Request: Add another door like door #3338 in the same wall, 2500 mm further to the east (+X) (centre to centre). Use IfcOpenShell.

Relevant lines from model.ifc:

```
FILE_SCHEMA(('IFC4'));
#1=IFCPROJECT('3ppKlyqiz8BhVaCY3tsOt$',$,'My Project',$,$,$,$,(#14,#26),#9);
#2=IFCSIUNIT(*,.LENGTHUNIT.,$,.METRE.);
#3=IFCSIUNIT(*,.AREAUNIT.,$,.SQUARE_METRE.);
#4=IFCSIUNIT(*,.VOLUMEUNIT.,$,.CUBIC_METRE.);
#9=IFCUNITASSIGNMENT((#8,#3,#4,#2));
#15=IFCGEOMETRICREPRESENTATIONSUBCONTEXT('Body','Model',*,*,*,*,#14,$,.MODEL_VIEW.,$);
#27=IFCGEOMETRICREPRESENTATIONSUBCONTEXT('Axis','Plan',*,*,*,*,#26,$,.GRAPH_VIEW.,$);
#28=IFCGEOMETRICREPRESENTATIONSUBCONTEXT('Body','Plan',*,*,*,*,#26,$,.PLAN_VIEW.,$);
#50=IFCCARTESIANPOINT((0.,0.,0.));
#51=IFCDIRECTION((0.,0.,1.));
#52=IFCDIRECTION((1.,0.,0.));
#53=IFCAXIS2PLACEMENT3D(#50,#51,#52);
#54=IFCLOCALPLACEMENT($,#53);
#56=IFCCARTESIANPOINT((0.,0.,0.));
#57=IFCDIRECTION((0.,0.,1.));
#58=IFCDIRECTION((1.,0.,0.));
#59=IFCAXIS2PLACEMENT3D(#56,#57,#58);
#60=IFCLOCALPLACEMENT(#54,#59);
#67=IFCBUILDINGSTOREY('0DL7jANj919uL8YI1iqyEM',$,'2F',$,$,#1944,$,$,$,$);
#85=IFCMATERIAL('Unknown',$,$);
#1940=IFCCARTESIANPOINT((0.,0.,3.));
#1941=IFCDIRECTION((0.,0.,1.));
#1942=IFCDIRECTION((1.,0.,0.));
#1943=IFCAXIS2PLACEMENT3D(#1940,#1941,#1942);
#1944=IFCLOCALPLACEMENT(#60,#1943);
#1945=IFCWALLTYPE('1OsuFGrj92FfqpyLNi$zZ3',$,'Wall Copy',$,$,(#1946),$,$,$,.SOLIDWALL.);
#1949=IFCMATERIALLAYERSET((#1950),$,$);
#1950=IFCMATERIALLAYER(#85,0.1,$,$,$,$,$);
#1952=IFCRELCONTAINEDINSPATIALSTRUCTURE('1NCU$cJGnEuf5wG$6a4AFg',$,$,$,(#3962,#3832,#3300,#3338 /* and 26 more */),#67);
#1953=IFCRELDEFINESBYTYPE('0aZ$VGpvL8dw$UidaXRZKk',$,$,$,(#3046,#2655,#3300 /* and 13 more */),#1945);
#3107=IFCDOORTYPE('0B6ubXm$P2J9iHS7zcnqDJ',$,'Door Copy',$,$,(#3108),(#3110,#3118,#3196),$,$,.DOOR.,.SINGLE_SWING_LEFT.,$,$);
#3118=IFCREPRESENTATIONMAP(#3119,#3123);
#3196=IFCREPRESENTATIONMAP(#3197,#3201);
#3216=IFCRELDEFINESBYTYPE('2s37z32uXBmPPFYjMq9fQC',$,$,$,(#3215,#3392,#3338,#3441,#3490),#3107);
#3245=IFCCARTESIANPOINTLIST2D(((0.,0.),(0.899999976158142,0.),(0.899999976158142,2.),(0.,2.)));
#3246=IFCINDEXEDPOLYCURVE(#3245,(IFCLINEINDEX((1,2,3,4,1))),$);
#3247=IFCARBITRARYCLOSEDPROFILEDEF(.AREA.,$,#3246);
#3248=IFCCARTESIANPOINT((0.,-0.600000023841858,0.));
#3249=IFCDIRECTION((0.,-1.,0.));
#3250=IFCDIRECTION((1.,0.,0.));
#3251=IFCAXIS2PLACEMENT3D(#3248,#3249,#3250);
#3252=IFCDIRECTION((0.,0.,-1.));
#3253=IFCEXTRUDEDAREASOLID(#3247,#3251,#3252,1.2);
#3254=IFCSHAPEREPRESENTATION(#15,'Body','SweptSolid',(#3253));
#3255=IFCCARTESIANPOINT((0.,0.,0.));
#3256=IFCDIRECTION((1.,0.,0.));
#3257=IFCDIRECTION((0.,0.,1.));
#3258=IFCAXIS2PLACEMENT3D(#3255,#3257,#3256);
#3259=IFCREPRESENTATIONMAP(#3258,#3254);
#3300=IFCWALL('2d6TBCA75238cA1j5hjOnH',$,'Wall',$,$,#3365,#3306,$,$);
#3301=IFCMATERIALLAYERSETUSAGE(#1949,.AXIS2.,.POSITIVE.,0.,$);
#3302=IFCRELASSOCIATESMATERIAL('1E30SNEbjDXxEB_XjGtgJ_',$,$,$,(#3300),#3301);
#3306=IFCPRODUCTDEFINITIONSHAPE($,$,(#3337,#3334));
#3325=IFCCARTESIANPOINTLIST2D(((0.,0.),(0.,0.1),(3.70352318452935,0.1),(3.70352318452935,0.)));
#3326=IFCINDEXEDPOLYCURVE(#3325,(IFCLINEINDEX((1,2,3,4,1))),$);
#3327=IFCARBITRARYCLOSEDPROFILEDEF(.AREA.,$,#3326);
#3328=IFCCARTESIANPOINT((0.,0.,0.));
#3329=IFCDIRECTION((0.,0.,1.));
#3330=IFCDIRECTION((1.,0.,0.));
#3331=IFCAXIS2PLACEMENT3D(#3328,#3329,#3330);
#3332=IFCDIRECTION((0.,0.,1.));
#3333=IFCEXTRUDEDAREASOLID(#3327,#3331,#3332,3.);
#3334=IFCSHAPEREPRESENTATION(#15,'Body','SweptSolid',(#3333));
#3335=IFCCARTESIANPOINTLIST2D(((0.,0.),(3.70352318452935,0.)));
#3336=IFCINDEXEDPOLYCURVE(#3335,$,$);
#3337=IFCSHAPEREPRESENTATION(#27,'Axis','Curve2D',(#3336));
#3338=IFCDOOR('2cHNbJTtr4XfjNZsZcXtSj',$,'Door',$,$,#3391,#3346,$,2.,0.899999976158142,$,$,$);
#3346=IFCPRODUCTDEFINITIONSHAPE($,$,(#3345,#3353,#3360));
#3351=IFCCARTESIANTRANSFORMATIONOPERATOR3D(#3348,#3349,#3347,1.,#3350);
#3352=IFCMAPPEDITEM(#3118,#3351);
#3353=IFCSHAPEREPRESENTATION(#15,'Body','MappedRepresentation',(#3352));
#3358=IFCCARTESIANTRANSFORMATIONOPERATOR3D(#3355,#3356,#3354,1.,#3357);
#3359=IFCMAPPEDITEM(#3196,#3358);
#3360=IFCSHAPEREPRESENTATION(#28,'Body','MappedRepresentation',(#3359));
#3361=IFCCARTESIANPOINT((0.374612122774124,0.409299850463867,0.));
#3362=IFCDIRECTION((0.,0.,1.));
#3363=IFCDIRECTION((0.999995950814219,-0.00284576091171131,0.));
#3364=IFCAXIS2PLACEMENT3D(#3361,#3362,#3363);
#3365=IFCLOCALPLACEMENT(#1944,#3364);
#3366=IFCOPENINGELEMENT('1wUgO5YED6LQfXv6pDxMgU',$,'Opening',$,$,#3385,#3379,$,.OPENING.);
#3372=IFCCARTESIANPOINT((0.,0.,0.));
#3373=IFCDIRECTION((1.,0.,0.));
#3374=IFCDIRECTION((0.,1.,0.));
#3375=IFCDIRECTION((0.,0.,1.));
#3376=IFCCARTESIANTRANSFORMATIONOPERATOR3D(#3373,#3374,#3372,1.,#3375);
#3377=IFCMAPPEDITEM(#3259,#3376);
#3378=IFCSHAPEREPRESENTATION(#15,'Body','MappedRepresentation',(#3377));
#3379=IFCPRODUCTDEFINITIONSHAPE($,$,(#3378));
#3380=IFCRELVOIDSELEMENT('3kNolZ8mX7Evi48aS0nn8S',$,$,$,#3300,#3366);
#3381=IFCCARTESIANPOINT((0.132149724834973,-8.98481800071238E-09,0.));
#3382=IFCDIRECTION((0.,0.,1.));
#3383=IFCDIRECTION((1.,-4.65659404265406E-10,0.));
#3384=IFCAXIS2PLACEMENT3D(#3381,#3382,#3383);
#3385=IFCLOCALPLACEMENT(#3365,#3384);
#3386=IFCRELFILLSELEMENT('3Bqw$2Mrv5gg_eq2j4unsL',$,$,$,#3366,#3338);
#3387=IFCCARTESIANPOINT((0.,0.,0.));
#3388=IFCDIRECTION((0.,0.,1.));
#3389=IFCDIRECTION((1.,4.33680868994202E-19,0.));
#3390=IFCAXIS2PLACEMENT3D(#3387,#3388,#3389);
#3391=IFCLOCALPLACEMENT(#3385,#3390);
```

```python
import ifcopenshell
import ifcopenshell.api.feature
import ifcopenshell.api.geometry
import ifcopenshell.api.root
import ifcopenshell.geom
import ifcopenshell.util.element
import ifcopenshell.util.placement
import ifcopenshell.util.shape

model = ifcopenshell.open("model.ifc")
settings = ifcopenshell.geom.settings()


def volume(element):
    """Net volume in cubic metres, openings subtracted."""
    shape = ifcopenshell.geom.create_shape(settings, element)
    return ifcopenshell.util.shape.get_volume(shape.geometry)


door = model.by_id(3338)
opening = door.FillsVoids[0].RelatingOpeningElement
wall = opening.VoidsElements[0].RelatingBuildingElement
before = volume(wall)
shift = ifcopenshell.util.placement.get_local_placement(wall.ObjectPlacement)[:3, 0] * 2.5

# copy_class copies the void relationship, type, container and properties, but no geometry.
new_opening = ifcopenshell.api.root.copy_class(model, product=opening)
new_opening.Representation = ifcopenshell.util.element.copy_deep(
    model, opening.Representation, exclude=["IfcGeometricRepresentationContext", "IfcRepresentationMap"]
)
new_door = ifcopenshell.api.root.copy_class(model, product=door)
new_door.Representation = ifcopenshell.util.element.copy_deep(
    model, door.Representation, exclude=["IfcGeometricRepresentationContext", "IfcRepresentationMap"]
)
ifcopenshell.api.feature.add_filling(model, opening=new_opening, element=new_door)

for old, new in ((opening, new_opening), (door, new_door)):
    matrix = ifcopenshell.util.placement.get_local_placement(old.ObjectPlacement)
    matrix[:3, 3] += shift
    ifcopenshell.api.geometry.edit_object_placement(model, product=new, matrix=matrix, is_si=False)

after = volume(wall)

print(f"wall volume {before:.3f} -> {after:.3f} m3")

model.write("model-out.ifc")
```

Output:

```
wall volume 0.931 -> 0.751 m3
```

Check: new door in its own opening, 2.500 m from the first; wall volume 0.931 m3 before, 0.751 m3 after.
